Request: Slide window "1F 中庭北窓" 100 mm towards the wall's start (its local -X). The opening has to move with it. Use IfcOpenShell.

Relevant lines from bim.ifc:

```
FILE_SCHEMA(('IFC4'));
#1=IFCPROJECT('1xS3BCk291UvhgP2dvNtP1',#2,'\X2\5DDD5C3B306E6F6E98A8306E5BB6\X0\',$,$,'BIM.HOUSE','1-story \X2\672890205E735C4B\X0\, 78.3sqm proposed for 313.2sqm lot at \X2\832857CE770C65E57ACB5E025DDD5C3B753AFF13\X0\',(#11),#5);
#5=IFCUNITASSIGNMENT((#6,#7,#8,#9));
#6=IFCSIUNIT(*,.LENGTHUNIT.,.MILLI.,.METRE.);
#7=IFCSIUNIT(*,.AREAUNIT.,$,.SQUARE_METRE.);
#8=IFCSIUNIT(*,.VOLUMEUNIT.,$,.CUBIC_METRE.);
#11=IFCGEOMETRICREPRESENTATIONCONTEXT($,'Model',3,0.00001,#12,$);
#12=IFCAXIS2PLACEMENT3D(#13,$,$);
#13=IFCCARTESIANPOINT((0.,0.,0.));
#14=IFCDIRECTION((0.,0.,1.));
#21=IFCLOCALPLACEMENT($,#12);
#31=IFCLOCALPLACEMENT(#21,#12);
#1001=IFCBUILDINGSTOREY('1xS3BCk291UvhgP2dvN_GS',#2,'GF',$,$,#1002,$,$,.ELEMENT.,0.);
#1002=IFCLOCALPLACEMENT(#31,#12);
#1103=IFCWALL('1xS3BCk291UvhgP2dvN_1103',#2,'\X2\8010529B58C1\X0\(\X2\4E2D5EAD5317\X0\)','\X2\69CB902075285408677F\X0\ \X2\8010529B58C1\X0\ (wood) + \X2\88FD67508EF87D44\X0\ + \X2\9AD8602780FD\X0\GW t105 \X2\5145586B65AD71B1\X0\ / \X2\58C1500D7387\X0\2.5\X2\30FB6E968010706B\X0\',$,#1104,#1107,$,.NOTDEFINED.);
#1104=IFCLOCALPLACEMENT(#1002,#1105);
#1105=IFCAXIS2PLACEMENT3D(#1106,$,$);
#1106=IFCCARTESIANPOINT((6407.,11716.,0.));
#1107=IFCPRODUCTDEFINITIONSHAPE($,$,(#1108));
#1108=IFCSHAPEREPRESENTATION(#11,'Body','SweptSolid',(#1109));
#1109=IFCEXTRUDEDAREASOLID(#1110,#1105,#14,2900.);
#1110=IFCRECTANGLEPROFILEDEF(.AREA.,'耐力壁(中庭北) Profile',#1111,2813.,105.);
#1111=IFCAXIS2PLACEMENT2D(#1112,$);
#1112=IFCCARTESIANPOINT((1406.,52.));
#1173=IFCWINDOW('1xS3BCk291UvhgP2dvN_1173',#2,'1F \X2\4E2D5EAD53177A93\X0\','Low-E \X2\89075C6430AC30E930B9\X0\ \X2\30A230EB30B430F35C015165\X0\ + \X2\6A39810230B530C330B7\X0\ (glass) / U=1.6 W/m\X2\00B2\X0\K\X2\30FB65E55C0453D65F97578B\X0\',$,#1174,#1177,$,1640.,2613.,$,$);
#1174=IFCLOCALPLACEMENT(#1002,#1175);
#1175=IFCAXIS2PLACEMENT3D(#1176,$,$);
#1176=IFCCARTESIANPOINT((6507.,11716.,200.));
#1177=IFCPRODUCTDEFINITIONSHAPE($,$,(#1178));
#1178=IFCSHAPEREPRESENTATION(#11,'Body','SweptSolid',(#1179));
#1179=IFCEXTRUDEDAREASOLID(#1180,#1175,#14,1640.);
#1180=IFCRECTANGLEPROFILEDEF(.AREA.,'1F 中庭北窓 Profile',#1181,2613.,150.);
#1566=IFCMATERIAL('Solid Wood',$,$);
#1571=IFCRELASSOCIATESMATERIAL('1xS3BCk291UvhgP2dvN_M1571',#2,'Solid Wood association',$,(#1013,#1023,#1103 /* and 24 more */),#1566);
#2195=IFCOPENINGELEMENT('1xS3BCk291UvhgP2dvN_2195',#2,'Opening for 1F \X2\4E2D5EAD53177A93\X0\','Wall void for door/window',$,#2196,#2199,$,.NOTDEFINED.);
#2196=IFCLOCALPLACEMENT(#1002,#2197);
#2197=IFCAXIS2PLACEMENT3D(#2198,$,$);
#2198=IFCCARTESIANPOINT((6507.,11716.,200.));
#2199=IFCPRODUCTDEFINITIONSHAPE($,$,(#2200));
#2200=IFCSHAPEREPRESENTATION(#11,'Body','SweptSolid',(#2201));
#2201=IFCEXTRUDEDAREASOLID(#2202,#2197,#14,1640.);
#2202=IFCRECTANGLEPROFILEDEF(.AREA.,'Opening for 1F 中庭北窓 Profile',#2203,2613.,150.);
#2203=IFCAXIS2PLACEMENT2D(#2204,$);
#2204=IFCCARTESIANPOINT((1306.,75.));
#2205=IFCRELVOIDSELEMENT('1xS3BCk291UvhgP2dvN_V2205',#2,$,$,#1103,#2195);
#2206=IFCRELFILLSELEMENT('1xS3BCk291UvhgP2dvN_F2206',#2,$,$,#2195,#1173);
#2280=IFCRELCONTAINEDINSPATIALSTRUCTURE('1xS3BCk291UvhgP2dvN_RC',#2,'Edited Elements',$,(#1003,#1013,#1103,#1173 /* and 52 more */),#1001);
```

```python
import ifcopenshell
import ifcopenshell.api.geometry
import ifcopenshell.util.placement
import ifcopenshell.util.unit

model = ifcopenshell.open("bim.ifc")
unit_scale = ifcopenshell.util.unit.calculate_unit_scale(model)

window = model.by_guid("1xS3BCk291UvhgP2dvN_1173")
opening = window.FillsVoids[0].RelatingOpeningElement
wall = opening.VoidsElements[0].RelatingBuildingElement

wall_matrix = ifcopenshell.util.placement.get_local_placement(wall.ObjectPlacement)
shift = wall_matrix[:3, 0] * -0.1 / unit_scale
before = ifcopenshell.util.placement.get_local_placement(window.ObjectPlacement)[:3, 3].copy()

# The window is not placed relative to its opening, so move both.
for product in (opening, window):
    matrix = ifcopenshell.util.placement.get_local_placement(product.ObjectPlacement)
    matrix[:3, 3] += shift
    ifcopenshell.api.geometry.edit_object_placement(model, product=product, matrix=matrix, is_si=False)

after = ifcopenshell.util.placement.get_local_placement(window.ObjectPlacement)[:3, 3]
print("window moved by", (after - before).round(3) + 0.0)

model.write("bim_updated.ifc")
```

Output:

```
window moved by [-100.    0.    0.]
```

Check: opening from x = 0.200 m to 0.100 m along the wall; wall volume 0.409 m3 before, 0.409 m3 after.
